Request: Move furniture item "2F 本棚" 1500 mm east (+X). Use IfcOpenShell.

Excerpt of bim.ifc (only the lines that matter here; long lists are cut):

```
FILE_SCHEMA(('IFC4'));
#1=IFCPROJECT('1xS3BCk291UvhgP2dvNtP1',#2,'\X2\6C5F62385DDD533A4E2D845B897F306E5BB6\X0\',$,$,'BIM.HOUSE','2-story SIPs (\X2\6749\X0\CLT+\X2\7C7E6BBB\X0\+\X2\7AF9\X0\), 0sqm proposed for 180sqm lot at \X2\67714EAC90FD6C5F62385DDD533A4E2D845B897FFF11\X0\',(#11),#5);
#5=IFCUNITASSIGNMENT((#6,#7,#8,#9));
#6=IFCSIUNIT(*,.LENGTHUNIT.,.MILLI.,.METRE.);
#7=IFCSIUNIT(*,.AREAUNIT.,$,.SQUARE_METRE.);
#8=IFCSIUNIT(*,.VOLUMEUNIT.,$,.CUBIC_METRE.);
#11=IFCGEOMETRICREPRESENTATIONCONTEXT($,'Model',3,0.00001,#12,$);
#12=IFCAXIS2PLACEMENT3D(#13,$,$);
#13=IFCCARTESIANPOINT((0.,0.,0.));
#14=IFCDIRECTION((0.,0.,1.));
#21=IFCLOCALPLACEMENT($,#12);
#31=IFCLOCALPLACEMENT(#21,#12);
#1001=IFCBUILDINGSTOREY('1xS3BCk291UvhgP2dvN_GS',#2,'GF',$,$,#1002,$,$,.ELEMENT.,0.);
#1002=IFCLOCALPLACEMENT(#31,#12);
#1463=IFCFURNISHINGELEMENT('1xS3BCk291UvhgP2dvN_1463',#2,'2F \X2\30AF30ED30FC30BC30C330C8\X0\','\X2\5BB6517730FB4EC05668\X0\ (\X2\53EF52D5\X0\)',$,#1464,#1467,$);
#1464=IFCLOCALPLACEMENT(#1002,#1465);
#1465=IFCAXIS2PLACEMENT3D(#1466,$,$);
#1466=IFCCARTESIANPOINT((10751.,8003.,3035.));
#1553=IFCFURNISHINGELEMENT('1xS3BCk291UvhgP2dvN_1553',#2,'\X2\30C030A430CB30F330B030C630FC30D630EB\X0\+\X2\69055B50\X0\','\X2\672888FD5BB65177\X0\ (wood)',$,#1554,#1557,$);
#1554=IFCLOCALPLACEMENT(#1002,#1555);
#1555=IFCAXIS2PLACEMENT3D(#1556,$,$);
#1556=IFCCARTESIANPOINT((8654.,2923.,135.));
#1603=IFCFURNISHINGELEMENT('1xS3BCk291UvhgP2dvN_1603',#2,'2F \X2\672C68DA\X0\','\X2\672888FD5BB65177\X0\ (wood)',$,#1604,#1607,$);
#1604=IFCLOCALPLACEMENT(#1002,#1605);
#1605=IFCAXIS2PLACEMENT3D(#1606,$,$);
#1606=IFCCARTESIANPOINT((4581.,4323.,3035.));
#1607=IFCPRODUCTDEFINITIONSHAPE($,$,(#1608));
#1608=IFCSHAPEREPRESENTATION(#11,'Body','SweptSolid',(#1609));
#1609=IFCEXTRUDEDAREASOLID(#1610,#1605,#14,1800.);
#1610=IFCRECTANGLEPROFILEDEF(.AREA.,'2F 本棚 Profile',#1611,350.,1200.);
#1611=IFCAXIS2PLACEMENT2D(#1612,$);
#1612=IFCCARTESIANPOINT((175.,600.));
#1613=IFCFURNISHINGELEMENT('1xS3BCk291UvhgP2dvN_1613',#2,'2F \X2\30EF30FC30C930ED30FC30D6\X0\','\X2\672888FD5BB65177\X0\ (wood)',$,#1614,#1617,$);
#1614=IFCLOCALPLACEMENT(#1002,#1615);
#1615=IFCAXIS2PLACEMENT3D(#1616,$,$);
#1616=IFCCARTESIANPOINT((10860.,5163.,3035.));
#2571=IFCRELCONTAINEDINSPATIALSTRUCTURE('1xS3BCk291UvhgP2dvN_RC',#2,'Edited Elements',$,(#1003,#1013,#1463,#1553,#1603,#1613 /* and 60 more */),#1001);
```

```python
import ifcopenshell
import ifcopenshell.api.geometry
import ifcopenshell.util.placement

model = ifcopenshell.open("bim.ifc")

item = model.by_guid("1xS3BCk291UvhgP2dvN_1603")
matrix = ifcopenshell.util.placement.get_local_placement(item.ObjectPlacement)
matrix[0, 3] += 1500.0
ifcopenshell.api.geometry.edit_object_placement(model, product=item, matrix=matrix, is_si=False)

print(ifcopenshell.util.placement.get_local_placement(item.ObjectPlacement).round(3) + 0.0)

model.write("bim_updated.ifc")
```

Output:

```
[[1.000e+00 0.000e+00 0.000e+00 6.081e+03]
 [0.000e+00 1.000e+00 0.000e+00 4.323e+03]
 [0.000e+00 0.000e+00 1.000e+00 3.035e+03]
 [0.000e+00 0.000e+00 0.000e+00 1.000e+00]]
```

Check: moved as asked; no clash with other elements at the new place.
